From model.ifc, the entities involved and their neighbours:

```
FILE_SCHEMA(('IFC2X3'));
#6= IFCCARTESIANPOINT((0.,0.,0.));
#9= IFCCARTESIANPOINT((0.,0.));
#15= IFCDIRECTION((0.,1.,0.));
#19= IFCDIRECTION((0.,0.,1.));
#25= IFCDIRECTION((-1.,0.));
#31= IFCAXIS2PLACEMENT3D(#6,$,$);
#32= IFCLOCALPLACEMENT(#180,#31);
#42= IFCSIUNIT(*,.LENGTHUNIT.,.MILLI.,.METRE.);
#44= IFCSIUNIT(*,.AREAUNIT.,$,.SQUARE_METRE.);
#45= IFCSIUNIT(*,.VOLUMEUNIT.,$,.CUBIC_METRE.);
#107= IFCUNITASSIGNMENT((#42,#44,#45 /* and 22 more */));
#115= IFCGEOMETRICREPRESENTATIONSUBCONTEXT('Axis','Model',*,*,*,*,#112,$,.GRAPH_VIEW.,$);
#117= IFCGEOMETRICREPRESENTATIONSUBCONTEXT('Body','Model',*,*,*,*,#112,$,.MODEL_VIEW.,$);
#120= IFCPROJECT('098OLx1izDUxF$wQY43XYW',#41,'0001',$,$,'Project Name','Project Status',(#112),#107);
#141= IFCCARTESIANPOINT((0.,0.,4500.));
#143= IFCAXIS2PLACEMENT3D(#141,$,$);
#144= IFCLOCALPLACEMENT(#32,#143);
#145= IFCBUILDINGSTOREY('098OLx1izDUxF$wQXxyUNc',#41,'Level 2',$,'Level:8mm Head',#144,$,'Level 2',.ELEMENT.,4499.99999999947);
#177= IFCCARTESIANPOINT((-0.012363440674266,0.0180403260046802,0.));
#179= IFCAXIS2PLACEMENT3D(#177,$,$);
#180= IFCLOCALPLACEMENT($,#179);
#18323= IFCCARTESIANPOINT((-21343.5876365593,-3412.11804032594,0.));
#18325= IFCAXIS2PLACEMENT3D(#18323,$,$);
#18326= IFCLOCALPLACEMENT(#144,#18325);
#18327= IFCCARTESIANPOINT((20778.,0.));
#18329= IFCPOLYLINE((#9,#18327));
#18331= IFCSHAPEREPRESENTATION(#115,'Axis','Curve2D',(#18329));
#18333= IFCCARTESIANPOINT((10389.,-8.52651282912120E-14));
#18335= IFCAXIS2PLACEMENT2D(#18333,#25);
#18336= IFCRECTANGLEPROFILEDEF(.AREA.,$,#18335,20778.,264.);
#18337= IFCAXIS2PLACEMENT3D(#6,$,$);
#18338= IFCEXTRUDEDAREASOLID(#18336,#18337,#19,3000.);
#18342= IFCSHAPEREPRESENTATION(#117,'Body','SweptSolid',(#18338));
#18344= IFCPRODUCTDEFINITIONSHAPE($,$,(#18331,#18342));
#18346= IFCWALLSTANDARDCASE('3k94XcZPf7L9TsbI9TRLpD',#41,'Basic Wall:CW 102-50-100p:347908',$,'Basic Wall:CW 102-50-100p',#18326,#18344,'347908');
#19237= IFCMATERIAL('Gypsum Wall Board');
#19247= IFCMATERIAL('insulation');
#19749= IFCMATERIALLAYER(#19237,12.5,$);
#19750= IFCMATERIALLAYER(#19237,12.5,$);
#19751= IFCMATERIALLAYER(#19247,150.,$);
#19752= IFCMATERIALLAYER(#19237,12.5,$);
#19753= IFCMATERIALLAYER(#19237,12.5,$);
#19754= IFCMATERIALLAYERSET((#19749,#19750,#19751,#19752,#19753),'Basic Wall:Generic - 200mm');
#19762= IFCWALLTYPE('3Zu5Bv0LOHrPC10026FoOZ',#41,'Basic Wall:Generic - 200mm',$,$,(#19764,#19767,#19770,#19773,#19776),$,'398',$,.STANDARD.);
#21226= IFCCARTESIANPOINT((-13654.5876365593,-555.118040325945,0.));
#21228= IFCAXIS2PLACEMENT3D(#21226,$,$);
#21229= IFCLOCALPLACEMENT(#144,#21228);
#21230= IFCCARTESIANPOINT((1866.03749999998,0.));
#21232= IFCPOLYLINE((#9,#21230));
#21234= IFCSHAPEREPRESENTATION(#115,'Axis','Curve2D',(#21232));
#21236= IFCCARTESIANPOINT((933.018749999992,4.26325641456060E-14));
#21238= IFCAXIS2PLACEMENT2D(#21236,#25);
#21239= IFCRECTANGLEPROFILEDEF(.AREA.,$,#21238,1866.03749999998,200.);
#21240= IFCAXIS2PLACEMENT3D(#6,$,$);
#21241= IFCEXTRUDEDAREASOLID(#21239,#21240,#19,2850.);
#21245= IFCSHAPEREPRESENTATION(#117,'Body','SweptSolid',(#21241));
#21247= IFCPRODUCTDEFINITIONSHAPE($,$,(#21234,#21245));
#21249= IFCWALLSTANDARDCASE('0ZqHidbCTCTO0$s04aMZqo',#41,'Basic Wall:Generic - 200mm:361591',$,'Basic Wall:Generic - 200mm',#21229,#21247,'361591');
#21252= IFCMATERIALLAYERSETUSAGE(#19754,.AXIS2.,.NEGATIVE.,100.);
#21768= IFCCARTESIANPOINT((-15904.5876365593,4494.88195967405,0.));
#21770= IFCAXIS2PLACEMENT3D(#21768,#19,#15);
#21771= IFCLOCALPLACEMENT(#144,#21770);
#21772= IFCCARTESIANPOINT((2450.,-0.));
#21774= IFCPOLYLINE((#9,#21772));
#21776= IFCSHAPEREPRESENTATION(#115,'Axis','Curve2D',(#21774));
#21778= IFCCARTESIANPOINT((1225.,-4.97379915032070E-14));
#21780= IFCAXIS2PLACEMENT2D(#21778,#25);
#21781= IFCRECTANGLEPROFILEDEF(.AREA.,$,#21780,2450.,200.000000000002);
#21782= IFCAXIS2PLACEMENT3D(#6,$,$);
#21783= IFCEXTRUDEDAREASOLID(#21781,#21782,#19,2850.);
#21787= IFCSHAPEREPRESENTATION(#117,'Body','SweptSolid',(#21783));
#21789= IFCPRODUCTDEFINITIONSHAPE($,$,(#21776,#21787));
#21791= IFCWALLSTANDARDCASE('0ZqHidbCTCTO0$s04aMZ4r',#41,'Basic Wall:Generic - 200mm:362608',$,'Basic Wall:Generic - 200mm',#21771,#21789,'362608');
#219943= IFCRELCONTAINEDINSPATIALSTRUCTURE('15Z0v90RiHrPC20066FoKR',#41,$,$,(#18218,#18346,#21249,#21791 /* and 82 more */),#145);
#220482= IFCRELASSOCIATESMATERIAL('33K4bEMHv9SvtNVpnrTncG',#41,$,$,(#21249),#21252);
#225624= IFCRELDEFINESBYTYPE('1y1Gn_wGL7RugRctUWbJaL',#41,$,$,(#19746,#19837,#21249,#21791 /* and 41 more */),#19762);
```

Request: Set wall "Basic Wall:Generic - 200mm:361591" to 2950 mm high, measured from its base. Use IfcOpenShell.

```python
import ifcopenshell
import ifcopenshell.geom
import ifcopenshell.util.representation
import ifcopenshell.util.shape
import ifcopenshell.util.unit

model = ifcopenshell.open("model.ifc")
unit_scale = ifcopenshell.util.unit.calculate_unit_scale(model)
settings = ifcopenshell.geom.settings()


def volume(element):
    """Net volume in cubic metres, openings subtracted."""
    shape = ifcopenshell.geom.create_shape(settings, element)
    return ifcopenshell.util.shape.get_volume(shape.geometry)


wall = model.by_guid("0ZqHidbCTCTO0$s04aMZqo")
before = volume(wall)

body = ifcopenshell.util.representation.get_representation(wall, "Model", "Body")
solid = body.Items[0]
old_height = solid.Depth
solid.Depth = 2.95 / unit_scale
after = volume(wall)

print(f"height {old_height:g} -> {solid.Depth:g}, volume {before:.3f} -> {after:.3f} m3")

model.write("model_rev.ifc")
```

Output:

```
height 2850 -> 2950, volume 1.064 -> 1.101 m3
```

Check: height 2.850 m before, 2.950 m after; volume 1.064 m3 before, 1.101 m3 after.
